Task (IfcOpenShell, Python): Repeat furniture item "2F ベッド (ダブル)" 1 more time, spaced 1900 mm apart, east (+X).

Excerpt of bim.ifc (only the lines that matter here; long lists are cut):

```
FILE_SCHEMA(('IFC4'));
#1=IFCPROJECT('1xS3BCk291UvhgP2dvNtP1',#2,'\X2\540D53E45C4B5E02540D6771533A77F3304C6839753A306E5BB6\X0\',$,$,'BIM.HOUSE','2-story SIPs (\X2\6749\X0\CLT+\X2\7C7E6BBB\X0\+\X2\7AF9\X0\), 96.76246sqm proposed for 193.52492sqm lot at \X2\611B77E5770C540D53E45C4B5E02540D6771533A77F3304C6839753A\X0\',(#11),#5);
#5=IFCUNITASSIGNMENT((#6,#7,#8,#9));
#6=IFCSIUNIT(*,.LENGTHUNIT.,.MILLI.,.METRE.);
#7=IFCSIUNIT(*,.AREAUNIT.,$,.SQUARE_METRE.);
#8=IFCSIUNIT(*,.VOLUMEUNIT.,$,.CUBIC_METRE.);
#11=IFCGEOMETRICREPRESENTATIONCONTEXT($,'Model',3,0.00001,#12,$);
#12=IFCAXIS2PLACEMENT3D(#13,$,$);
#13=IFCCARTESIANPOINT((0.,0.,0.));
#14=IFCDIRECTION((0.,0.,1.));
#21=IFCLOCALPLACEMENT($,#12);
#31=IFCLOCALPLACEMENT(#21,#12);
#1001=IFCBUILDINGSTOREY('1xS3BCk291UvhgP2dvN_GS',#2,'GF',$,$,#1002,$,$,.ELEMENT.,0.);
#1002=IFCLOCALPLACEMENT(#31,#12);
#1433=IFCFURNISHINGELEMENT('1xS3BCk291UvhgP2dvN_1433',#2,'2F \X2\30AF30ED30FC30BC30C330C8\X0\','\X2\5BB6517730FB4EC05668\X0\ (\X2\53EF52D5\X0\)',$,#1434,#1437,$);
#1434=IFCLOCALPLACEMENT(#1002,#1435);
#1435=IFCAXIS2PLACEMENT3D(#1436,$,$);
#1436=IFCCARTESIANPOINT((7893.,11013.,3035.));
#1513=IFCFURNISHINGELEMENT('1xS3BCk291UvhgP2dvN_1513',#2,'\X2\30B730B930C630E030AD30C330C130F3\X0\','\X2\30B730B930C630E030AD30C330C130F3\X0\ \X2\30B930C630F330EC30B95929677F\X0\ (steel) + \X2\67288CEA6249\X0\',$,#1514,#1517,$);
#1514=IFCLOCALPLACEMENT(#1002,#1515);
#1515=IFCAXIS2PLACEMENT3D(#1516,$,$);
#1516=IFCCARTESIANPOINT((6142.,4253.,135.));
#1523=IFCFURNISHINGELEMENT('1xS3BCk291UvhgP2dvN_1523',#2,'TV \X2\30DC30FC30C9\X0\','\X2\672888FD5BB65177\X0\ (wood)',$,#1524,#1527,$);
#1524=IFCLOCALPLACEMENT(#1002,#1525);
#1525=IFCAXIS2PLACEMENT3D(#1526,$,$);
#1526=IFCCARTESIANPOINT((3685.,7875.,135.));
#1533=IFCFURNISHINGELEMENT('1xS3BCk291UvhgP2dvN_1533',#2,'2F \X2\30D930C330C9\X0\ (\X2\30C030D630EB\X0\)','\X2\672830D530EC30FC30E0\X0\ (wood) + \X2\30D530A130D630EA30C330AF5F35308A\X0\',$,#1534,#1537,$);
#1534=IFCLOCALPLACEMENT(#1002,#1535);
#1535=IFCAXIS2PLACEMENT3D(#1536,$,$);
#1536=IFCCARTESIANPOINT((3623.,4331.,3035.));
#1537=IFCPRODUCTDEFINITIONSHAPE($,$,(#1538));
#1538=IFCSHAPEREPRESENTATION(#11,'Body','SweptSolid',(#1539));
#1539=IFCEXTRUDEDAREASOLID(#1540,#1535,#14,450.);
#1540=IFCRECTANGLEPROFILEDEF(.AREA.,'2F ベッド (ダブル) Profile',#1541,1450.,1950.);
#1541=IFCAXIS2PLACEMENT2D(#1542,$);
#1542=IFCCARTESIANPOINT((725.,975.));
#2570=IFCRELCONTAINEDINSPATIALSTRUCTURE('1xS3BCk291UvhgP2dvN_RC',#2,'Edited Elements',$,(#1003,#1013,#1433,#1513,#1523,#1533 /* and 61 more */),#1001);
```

```python
import numpy as np
import ifcopenshell
import ifcopenshell.api.geometry
import ifcopenshell.api.root
import ifcopenshell.util.element
import ifcopenshell.util.placement
import ifcopenshell.util.unit

model = ifcopenshell.open("bim.ifc")
unit_scale = ifcopenshell.util.unit.calculate_unit_scale(model)


def reuse_history(source, copy):
    """copy_class also copies each property set's owner history, people and application; keep the originals."""
    for rel in copy.IsDefinedBy:
        if rel.is_a("IfcRelDefinesByProperties") and (history := rel.RelatingPropertyDefinition.OwnerHistory):
            rel.RelatingPropertyDefinition.OwnerHistory = source.OwnerHistory
            ifcopenshell.util.element.remove_deep2(model, history)


source = model.by_guid("1xS3BCk291UvhgP2dvN_1533")
base = ifcopenshell.util.placement.get_local_placement(source.ObjectPlacement)
step = np.array([1.0, 0.0, 0.0]) * 1.9 / unit_scale

for i in range(1, 2):
    copy = ifcopenshell.api.root.copy_class(model, product=source)
    copy.Representation = ifcopenshell.util.element.copy_deep(
        model, source.Representation, exclude=["IfcGeometricRepresentationContext", "IfcRepresentationMap"]
    )
    reuse_history(source, copy)
    matrix = base.copy()
    matrix[:3, 3] += i * step
    print("added at", matrix[:3, 3].round(3) + 0.0)
    ifcopenshell.api.geometry.edit_object_placement(model, product=copy, matrix=matrix, is_si=False)

model.write("bim_rev.ifc")
```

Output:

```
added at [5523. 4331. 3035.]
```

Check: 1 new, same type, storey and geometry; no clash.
